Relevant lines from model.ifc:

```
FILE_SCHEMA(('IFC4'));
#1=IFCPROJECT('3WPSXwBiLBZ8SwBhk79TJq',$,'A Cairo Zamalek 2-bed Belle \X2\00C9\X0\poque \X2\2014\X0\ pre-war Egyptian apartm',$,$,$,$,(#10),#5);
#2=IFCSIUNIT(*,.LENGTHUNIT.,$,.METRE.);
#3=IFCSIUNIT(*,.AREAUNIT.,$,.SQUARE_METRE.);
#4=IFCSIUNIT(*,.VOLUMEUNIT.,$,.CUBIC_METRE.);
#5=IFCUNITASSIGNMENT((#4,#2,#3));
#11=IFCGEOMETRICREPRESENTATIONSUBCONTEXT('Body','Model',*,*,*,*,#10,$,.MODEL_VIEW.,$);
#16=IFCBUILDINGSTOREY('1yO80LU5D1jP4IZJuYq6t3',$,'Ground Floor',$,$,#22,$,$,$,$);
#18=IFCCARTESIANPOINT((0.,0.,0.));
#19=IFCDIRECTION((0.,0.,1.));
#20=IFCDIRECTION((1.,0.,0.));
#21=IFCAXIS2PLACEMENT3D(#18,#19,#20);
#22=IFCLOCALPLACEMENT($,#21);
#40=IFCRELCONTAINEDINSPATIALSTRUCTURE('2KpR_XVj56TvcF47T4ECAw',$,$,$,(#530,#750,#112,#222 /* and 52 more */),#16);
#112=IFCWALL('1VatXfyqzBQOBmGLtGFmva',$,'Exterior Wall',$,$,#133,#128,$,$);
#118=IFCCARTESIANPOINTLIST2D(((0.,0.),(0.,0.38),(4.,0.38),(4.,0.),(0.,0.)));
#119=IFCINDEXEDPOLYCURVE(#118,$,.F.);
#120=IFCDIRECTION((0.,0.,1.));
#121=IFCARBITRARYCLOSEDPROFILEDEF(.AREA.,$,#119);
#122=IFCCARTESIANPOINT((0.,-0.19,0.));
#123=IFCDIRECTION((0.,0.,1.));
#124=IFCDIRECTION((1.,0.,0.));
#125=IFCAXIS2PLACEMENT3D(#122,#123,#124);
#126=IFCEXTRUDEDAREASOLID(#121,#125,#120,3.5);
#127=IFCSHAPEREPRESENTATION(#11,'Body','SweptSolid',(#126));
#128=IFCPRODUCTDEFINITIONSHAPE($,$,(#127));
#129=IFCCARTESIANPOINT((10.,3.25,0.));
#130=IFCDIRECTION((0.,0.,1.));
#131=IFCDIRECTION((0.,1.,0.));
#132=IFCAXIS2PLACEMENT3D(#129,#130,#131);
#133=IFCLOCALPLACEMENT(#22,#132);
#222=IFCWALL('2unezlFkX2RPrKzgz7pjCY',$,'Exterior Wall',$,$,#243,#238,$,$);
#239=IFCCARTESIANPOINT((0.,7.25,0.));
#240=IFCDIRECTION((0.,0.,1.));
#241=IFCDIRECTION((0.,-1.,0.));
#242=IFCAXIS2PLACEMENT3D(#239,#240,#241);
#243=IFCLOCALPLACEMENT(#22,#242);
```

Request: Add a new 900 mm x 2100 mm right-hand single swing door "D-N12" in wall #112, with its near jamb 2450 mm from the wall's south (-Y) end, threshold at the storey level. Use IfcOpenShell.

```python
import numpy as np
import ifcopenshell
import ifcopenshell.api.feature
import ifcopenshell.api.geometry
import ifcopenshell.api.root
import ifcopenshell.api.spatial
import ifcopenshell.geom
import ifcopenshell.util.element
import ifcopenshell.util.placement
import ifcopenshell.util.representation
import ifcopenshell.util.shape
import ifcopenshell.util.unit

model = ifcopenshell.open("model.ifc")
unit_scale = ifcopenshell.util.unit.calculate_unit_scale(model)
settings = ifcopenshell.geom.settings()


def volume(element):
    """Net volume in cubic metres, openings subtracted."""
    shape = ifcopenshell.geom.create_shape(settings, element)
    return ifcopenshell.util.shape.get_volume(shape.geometry)


wall = model.by_id(112)
storey = ifcopenshell.util.element.get_container(wall, ifc_class="IfcBuildingStorey")
context = ifcopenshell.util.representation.get_context(model, "Model", "Body", "MODEL_VIEW")
before = volume(wall)

width, height, from_end, sill = 0.9, 2.1, 2.45, 0.0  # metres

# The wall runs along its own X axis, and the end named is its -X end.
wall_shape = ifcopenshell.geom.create_shape(settings, wall)
x, y, z = ifcopenshell.util.shape.get_vertices(wall_shape.geometry).T
start = x.min() + from_end
face, thickness = float(y.min()), float(y.max() - y.min())
wall_matrix = ifcopenshell.util.placement.get_local_placement(wall.ObjectPlacement)
level = ifcopenshell.util.placement.get_local_placement(storey.ObjectPlacement)[2, 3]


def in_wall(x, y):
    """Placement at x, y metres in the wall's axes, at sill height."""
    matrix = wall_matrix.copy()
    matrix[:, 3] = wall_matrix @ np.array([x / unit_scale, y / unit_scale, 0.0, 1.0])
    matrix[2, 3] = level + sill / unit_scale
    return matrix


# Opening: a box that overshoots both wall faces by 50 mm.
opening = ifcopenshell.api.root.create_entity(model, ifc_class="IfcOpeningElement", predefined_type="OPENING")
box = ifcopenshell.api.geometry.add_wall_representation(
    model, context=context, length=width, height=height, thickness=thickness + 0.1
)
ifcopenshell.api.geometry.assign_representation(model, product=opening, representation=box)
ifcopenshell.api.geometry.edit_object_placement(model, product=opening, matrix=in_wall(start, face - 0.05), is_si=False)
ifcopenshell.api.feature.add_feature(model, feature=opening, element=wall)

door = ifcopenshell.api.root.create_entity(model, ifc_class="IfcDoor", name="D-N12", predefined_type="DOOR")
door.OverallWidth, door.OverallHeight = width / unit_scale, height / unit_scale
door.OperationType = "SINGLE_SWING_RIGHT"
body = ifcopenshell.api.geometry.add_door_representation(
    model,
    context=context,
    overall_width=door.OverallWidth,
    overall_height=door.OverallHeight,
    operation_type="SINGLE_SWING_RIGHT",
    lining_properties={"LiningDepth": thickness / unit_scale, "ThresholdDepth": thickness / unit_scale},
)
ifcopenshell.api.geometry.assign_representation(model, product=door, representation=body)
ifcopenshell.api.spatial.assign_container(model, products=[door], relating_structure=storey)
ifcopenshell.api.feature.add_filling(model, opening=opening, element=door)

# The lining spans the wall, so the door starts at the wall face.
ifcopenshell.api.geometry.edit_object_placement(model, product=door, matrix=in_wall(start, face), is_si=False)

after = volume(wall)

print(f"wall volume {before:.3f} -> {after:.3f} m3")

model.write("model_updated.ifc")
```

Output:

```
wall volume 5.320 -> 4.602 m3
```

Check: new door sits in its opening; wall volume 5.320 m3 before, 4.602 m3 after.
